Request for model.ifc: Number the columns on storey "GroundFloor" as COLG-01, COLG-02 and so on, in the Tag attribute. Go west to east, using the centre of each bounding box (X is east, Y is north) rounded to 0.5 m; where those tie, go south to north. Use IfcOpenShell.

First a look at what the model holds.

```python
import ifcopenshell
import ifcopenshell.util.element
import ifcopenshell.util.placement

model = ifcopenshell.open("model.ifc")
print(model.schema)
storey = next(s for s in model.by_type("IfcBuildingStorey") if s.Name == "GroundFloor")
columns = [e for e in ifcopenshell.util.element.get_decomposition(storey) if e.is_a("IfcColumn")]
for e in sorted(columns, key=lambda e: e.id()):
    origin = ifcopenshell.util.placement.get_local_placement(e.ObjectPlacement)[:3, 3]
    print(e.id(), e.Tag, e.Name, origin.round(2) + 0.0, sep=" | ")
```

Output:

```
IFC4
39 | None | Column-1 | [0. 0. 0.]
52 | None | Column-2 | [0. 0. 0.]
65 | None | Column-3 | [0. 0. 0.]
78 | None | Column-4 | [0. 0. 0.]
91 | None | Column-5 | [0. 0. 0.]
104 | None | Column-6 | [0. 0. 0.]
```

```python
import ifcopenshell
import ifcopenshell.geom
import ifcopenshell.util.element
import ifcopenshell.util.shape

model = ifcopenshell.open("model.ifc")
settings = ifcopenshell.geom.settings()
settings.set("use-world-coords", True)


def centre(element):
    shape = ifcopenshell.geom.create_shape(settings, element)
    return ifcopenshell.util.shape.get_bbox_centroid(shape.geometry)


storey = next(s for s in model.by_type("IfcBuildingStorey") if s.Name == "GroundFloor")
columns = [e for e in ifcopenshell.util.element.get_decomposition(storey) if e.is_a("IfcColumn")]

# Insertion points can sit at a corner or the storey origin, so sort by the geometry (in metres).
centres = {e: centre(e) for e in columns}
columns.sort(key=lambda e: (round(centres[e][0] / 0.5), centres[e][1]))

for i, e in enumerate(columns, start=1):
    number = f"COLG-{i:02d}"
    e.Tag = number
    print(e.id(), number)

model.write("model_edited.ifc")
```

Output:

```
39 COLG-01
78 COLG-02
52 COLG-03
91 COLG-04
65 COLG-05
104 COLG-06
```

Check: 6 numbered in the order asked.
